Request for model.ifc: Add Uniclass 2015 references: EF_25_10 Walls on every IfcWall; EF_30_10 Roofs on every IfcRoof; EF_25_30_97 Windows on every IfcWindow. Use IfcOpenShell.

First a look at what the model holds.

```python
import ifcopenshell

model = ifcopenshell.open("model.ifc")
print(model.schema)
print("classifications:", [c.Name for c in model.by_type("IfcClassification")])
for ifc_class in ("IfcDoor", "IfcRoof", "IfcStair", "IfcWall", "IfcWindow"):
    print(ifc_class, len(model.by_type(ifc_class)))
```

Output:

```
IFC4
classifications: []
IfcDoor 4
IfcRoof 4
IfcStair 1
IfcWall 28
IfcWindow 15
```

```python
import ifcopenshell
import ifcopenshell.api.classification

model = ifcopenshell.open("model.ifc")

system = ifcopenshell.api.classification.add_classification(model, classification="Uniclass 2015")

codes = {
    "IfcWall": ("EF_25_10", "Walls"),
    "IfcRoof": ("EF_30_10", "Roofs"),
    "IfcWindow": ("EF_25_30_97", "Windows"),
}
for ifc_class, (code, name) in codes.items():
    products = model.by_type(ifc_class)
    ifcopenshell.api.classification.add_reference(
        model, products=products, classification=system, identification=code, name=name
    )
    print(code, len(products))

model.write("model_updated.ifc")
```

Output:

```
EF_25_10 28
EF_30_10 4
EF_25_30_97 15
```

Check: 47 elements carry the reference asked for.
